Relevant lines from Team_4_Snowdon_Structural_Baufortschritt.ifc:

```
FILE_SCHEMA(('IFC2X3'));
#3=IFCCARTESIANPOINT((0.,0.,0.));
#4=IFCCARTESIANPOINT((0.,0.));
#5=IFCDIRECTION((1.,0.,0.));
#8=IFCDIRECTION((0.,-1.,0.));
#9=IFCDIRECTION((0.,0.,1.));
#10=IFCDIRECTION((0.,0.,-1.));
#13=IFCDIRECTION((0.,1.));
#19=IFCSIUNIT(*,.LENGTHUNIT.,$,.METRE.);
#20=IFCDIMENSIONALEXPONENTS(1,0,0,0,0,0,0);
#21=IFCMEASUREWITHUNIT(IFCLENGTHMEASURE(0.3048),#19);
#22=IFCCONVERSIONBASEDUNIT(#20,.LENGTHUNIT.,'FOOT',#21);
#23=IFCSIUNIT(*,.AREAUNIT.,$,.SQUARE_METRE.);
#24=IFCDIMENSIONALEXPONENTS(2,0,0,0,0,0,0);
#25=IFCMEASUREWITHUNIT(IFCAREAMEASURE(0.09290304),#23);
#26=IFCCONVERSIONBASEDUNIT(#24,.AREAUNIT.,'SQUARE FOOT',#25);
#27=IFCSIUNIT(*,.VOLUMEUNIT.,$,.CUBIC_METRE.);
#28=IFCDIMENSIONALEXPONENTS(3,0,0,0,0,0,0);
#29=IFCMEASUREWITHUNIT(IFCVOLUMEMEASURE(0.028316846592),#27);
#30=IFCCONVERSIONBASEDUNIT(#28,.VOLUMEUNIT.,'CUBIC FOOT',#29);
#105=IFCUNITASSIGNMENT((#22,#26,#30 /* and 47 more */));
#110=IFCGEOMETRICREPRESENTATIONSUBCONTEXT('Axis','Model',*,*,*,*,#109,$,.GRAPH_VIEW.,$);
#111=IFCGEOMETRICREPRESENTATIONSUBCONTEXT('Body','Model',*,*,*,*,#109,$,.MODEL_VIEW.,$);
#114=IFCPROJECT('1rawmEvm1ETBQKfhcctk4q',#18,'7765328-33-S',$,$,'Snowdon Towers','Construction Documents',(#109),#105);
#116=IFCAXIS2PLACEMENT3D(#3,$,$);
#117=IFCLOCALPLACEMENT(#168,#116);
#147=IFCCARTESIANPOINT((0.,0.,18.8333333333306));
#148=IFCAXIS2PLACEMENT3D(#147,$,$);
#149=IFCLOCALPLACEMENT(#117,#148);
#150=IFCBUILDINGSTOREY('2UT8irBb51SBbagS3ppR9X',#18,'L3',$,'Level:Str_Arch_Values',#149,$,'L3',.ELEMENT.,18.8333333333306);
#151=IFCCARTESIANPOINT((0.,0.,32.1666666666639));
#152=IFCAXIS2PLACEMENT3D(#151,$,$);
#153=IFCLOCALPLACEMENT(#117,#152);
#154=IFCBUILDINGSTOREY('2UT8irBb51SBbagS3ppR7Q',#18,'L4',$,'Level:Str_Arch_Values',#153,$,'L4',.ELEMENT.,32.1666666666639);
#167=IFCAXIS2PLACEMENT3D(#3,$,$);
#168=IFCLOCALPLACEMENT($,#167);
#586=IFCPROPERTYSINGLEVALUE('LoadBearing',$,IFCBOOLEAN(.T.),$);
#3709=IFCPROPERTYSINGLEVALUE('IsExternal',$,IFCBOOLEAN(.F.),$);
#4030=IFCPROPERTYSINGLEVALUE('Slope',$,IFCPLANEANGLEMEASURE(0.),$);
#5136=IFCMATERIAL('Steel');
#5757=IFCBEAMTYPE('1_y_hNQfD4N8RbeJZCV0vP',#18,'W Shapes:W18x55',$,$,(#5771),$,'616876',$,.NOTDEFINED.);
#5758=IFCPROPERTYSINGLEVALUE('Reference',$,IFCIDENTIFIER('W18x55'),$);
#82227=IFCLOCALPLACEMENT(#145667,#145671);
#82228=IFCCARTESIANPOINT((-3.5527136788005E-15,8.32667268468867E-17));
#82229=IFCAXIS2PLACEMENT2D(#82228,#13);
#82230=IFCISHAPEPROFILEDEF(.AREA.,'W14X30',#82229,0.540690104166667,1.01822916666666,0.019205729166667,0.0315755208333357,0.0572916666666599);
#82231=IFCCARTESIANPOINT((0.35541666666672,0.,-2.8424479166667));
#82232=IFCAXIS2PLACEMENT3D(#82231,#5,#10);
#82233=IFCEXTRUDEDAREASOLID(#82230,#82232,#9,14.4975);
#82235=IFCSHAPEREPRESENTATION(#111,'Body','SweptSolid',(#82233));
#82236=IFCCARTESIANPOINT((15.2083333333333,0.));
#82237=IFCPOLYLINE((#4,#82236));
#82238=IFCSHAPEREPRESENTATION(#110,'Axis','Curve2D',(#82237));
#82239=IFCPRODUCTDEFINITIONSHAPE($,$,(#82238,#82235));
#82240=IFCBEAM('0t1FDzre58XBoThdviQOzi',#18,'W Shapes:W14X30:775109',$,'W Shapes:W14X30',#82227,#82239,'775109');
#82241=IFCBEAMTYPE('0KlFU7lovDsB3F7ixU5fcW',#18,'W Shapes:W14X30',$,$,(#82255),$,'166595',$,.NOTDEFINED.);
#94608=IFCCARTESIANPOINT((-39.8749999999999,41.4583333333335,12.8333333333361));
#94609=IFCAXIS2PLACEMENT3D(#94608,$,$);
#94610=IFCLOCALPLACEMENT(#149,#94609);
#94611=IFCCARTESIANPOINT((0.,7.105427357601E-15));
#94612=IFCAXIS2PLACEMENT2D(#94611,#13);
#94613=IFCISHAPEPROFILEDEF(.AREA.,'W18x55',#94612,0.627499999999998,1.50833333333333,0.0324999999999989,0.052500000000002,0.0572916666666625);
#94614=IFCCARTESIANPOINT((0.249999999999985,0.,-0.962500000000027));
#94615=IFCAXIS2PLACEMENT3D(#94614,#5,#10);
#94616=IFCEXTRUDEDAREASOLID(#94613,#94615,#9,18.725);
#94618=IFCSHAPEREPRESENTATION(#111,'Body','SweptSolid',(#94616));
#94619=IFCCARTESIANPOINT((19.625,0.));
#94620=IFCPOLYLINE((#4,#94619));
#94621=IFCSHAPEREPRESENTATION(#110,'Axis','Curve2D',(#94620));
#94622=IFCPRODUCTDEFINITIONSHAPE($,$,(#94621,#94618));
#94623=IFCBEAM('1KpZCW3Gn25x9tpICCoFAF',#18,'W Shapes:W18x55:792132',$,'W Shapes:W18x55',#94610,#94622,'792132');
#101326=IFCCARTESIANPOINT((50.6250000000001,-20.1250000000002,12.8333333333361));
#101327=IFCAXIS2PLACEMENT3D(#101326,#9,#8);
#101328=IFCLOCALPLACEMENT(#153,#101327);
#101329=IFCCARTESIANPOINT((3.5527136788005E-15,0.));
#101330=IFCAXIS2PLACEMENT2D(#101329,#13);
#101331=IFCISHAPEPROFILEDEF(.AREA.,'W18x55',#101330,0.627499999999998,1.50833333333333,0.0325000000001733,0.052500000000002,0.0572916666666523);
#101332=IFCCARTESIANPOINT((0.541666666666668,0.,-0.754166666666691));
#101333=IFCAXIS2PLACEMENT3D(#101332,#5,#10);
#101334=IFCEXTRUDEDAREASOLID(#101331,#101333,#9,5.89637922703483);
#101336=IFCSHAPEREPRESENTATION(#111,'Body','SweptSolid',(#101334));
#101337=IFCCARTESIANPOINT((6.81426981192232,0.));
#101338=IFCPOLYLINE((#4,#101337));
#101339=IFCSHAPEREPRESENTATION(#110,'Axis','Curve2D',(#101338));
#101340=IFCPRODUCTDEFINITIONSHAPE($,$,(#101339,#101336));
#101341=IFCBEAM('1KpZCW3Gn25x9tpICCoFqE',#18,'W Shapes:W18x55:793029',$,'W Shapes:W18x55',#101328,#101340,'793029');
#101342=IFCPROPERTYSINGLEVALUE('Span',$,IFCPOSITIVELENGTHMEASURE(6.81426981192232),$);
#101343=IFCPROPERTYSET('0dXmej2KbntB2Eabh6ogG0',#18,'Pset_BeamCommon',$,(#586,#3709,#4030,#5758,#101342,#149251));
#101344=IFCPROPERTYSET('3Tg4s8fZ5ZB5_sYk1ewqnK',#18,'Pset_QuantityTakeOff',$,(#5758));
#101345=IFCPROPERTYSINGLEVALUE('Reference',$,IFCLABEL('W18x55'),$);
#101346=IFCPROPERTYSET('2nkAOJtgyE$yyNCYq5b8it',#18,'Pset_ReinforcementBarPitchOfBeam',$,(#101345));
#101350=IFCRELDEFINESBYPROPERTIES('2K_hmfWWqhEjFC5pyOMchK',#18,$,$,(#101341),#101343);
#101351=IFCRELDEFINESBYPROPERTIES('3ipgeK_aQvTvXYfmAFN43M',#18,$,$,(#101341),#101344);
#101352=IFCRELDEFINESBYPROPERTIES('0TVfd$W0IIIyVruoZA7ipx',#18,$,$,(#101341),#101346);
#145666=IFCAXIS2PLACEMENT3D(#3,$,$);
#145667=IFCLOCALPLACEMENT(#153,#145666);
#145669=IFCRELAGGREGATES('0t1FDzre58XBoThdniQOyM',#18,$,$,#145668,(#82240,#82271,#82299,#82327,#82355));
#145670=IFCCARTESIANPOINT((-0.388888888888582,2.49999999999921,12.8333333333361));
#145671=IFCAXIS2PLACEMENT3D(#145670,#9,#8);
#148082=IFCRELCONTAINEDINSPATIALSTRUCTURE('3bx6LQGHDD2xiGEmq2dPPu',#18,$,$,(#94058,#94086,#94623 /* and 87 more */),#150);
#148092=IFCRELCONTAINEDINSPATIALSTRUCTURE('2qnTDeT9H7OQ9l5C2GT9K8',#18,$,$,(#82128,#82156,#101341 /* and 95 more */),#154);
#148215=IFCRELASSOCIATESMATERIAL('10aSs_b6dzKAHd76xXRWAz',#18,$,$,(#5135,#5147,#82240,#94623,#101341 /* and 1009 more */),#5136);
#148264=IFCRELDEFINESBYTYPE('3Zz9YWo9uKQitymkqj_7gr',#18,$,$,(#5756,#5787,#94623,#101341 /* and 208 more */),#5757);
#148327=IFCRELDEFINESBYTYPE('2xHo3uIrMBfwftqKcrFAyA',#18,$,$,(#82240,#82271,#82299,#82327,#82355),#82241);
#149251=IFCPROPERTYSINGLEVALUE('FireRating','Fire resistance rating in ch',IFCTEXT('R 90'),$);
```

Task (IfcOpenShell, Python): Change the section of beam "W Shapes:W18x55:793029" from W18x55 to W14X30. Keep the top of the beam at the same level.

```python
import ifcopenshell
import ifcopenshell.api.pset
import ifcopenshell.api.type
import ifcopenshell.util.element
import ifcopenshell.util.representation

model = ifcopenshell.open("Team_4_Snowdon_Structural_Baufortschritt.ifc")

member = model.by_guid("1KpZCW3Gn25x9tpICCoFqE")
source = next(p for p in model.by_type("IfcIShapeProfileDef") if p.ProfileName == "W14X30")

body = ifcopenshell.util.representation.get_representation(member, "Model", "Body")
solid = body.Items[0]
old_profile = solid.SweptArea

# Copy the section's sizes but keep this member's own profile position.
profile = ifcopenshell.util.element.copy(model, source)
# Profiles are centred, so shift by half the change in depth to hold the top.
shift = (old_profile.OverallDepth - profile.OverallDepth) / 2
x, y = old_profile.Position.Location.Coordinates
up = (-1.0, 0.0)  # upwards, in the solid's own plane
location = model.createIfcCartesianPoint((x + up[0] * shift, y + up[1] * shift))
profile.Position = model.createIfcAxis2Placement2D(location, old_profile.Position.RefDirection)
solid.SweptArea = profile
if not model.get_total_inverses(old_profile):
    ifcopenshell.util.element.remove_deep2(model, old_profile)

new_type = model.by_id(82241)
ifcopenshell.api.type.assign_type(
    model, related_objects=[member], relating_type=new_type, should_map_representations=False
)
member.Name = member.Name.replace("W18x55", "W14X30")
member.ObjectType = "W Shapes:W14X30"
pset = model.by_id(ifcopenshell.util.element.get_pset(member, "Pset_BeamCommon", should_inherit=False)["id"])
ifcopenshell.api.pset.edit_pset(model, pset=pset, properties={"Reference": "W14X30"})
pset = model.by_id(ifcopenshell.util.element.get_pset(member, "Pset_QuantityTakeOff", should_inherit=False)["id"])
ifcopenshell.api.pset.edit_pset(model, pset=pset, properties={"Reference": "W14X30"})
pset = model.by_id(ifcopenshell.util.element.get_pset(member, "Pset_ReinforcementBarPitchOfBeam", should_inherit=False)["id"])
ifcopenshell.api.pset.edit_pset(model, pset=pset, properties={"Reference": "W14X30"})

print(solid.SweptArea)

model.write("Team_4_Snowdon_Structural_Baufortschritt_updated.ifc")
```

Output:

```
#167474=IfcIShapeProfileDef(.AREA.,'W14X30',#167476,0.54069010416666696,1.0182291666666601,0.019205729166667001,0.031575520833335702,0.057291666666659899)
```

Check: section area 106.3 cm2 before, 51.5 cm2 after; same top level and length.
